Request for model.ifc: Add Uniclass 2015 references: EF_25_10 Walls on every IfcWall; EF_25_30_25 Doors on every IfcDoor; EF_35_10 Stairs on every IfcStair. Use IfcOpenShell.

First a look at what the model holds.

```python
import ifcopenshell

model = ifcopenshell.open("model.ifc")
print(model.schema)
print("classifications:", [c.Name for c in model.by_type("IfcClassification")])
for ifc_class in ("IfcDoor", "IfcRoof", "IfcStair", "IfcWall", "IfcWindow"):
    print(ifc_class, len(model.by_type(ifc_class)))
```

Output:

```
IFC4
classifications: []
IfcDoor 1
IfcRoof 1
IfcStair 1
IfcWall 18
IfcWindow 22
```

```python
import ifcopenshell
import ifcopenshell.api.classification

model = ifcopenshell.open("model.ifc")

system = ifcopenshell.api.classification.add_classification(model, classification="Uniclass 2015")

codes = {
    "IfcWall": ("EF_25_10", "Walls"),
    "IfcDoor": ("EF_25_30_25", "Doors"),
    "IfcStair": ("EF_35_10", "Stairs"),
}
for ifc_class, (code, name) in codes.items():
    products = model.by_type(ifc_class)
    ifcopenshell.api.classification.add_reference(
        model, products=products, classification=system, identification=code, name=name
    )
    print(code, len(products))

model.write("model_edited.ifc")
```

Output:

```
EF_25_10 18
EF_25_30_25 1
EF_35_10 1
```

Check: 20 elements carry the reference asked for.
